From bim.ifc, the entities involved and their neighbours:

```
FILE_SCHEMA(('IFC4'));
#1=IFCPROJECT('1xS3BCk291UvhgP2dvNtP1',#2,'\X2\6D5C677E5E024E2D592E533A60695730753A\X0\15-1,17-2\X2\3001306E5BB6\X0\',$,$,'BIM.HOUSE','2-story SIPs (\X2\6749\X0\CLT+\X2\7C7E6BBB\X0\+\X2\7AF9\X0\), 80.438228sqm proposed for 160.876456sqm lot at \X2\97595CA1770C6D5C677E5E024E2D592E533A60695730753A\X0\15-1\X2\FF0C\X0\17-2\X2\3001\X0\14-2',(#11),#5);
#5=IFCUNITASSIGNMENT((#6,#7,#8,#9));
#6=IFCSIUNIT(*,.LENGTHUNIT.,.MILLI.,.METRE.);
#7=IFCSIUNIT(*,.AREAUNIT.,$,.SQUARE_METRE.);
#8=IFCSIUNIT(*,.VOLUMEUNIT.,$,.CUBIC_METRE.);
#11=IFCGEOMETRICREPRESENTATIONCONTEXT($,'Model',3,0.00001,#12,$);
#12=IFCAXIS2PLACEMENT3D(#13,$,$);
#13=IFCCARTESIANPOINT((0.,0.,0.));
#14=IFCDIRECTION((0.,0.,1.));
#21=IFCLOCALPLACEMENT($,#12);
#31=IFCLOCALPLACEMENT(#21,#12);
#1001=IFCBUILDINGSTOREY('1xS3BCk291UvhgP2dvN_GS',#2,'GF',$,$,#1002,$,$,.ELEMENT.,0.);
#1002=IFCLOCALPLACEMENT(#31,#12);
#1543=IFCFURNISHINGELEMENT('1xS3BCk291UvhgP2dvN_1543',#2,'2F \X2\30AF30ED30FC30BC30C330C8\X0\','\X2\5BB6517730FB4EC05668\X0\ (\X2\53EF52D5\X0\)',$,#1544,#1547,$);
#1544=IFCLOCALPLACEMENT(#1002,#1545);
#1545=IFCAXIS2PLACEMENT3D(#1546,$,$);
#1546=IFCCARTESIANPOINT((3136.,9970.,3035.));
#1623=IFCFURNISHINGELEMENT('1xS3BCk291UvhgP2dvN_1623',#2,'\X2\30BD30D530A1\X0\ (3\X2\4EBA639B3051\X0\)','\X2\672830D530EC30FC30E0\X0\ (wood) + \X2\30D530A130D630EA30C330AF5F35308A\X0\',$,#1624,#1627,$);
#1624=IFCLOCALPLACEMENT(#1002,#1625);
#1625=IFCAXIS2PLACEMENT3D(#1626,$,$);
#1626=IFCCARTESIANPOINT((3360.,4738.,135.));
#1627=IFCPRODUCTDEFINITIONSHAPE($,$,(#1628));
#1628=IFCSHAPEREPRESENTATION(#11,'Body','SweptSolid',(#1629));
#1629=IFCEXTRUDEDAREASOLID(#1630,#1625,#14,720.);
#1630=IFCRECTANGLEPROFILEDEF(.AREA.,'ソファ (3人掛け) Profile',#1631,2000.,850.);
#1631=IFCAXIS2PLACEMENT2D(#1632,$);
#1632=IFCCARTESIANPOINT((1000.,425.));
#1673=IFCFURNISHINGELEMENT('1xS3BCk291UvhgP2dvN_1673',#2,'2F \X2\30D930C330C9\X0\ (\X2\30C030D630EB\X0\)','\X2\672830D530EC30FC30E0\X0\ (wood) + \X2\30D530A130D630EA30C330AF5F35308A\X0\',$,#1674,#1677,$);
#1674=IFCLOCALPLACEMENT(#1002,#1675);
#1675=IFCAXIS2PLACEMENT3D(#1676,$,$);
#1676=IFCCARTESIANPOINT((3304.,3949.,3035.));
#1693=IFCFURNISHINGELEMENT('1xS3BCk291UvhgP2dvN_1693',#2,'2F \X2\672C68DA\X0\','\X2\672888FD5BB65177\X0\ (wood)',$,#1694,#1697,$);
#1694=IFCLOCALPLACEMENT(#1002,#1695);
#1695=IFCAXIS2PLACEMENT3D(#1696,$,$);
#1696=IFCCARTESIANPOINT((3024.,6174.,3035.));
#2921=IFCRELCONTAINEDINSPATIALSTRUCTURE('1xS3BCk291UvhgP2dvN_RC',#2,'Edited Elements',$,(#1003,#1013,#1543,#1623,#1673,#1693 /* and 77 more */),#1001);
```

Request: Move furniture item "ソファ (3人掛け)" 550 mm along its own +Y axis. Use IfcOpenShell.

```python
import ifcopenshell
import ifcopenshell.api.geometry
import ifcopenshell.util.placement

model = ifcopenshell.open("bim.ifc")

item = model.by_guid("1xS3BCk291UvhgP2dvN_1623")
matrix = ifcopenshell.util.placement.get_local_placement(item.ObjectPlacement)
matrix[:3, 3] += matrix[:3, 1] * 550.0
ifcopenshell.api.geometry.edit_object_placement(model, product=item, matrix=matrix, is_si=False)

print(ifcopenshell.util.placement.get_local_placement(item.ObjectPlacement).round(3) + 0.0)

model.write("bim_rev.ifc")
```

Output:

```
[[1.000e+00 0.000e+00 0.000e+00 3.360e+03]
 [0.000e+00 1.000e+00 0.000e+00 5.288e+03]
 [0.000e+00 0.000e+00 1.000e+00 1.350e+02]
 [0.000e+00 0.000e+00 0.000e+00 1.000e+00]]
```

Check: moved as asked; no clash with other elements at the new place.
